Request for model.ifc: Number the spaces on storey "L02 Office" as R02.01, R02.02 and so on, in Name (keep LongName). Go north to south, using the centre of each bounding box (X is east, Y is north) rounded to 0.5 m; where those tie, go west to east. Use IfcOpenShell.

First a look at what the model holds.

```python
import ifcopenshell
import ifcopenshell.util.element
import ifcopenshell.util.placement

model = ifcopenshell.open("model.ifc")
print(model.schema)
storey = next(s for s in model.by_type("IfcBuildingStorey") if s.Name == "L02 Office")
spaces = [e for e in ifcopenshell.util.element.get_decomposition(storey) if e.is_a("IfcSpace")]
for e in sorted(spaces, key=lambda e: e.id()):
    origin = ifcopenshell.util.placement.get_local_placement(e.ObjectPlacement)[:3, 3]
    print(e.id(), e.Name, e.LongName, origin.round(2) + 0.0, sep=" | ")
```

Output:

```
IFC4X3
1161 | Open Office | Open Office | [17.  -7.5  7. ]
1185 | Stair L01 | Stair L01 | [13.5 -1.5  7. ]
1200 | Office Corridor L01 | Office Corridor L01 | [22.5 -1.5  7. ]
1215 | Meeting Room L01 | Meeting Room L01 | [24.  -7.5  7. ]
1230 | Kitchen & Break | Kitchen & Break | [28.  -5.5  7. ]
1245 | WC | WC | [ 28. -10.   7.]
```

```python
import ifcopenshell
import ifcopenshell.geom
import ifcopenshell.util.element
import ifcopenshell.util.shape

model = ifcopenshell.open("model.ifc")
settings = ifcopenshell.geom.settings()
settings.set("use-world-coords", True)


def centre(element):
    shape = ifcopenshell.geom.create_shape(settings, element)
    return ifcopenshell.util.shape.get_bbox_centroid(shape.geometry)


storey = next(s for s in model.by_type("IfcBuildingStorey") if s.Name == "L02 Office")
spaces = [e for e in ifcopenshell.util.element.get_decomposition(storey) if e.is_a("IfcSpace")]

# Insertion points can sit at a corner or the storey origin, so sort by the geometry (in metres).
centres = {e: centre(e) for e in spaces}
spaces.sort(key=lambda e: (-round(centres[e][1] / 0.5), centres[e][0]))

for i, e in enumerate(spaces, start=1):
    number = f"R02.{i:02d}"
    e.Name = number
    print(e.id(), number)

model.write("model-out.ifc")
```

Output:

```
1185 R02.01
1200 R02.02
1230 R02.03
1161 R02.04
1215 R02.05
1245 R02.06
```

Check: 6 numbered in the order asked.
